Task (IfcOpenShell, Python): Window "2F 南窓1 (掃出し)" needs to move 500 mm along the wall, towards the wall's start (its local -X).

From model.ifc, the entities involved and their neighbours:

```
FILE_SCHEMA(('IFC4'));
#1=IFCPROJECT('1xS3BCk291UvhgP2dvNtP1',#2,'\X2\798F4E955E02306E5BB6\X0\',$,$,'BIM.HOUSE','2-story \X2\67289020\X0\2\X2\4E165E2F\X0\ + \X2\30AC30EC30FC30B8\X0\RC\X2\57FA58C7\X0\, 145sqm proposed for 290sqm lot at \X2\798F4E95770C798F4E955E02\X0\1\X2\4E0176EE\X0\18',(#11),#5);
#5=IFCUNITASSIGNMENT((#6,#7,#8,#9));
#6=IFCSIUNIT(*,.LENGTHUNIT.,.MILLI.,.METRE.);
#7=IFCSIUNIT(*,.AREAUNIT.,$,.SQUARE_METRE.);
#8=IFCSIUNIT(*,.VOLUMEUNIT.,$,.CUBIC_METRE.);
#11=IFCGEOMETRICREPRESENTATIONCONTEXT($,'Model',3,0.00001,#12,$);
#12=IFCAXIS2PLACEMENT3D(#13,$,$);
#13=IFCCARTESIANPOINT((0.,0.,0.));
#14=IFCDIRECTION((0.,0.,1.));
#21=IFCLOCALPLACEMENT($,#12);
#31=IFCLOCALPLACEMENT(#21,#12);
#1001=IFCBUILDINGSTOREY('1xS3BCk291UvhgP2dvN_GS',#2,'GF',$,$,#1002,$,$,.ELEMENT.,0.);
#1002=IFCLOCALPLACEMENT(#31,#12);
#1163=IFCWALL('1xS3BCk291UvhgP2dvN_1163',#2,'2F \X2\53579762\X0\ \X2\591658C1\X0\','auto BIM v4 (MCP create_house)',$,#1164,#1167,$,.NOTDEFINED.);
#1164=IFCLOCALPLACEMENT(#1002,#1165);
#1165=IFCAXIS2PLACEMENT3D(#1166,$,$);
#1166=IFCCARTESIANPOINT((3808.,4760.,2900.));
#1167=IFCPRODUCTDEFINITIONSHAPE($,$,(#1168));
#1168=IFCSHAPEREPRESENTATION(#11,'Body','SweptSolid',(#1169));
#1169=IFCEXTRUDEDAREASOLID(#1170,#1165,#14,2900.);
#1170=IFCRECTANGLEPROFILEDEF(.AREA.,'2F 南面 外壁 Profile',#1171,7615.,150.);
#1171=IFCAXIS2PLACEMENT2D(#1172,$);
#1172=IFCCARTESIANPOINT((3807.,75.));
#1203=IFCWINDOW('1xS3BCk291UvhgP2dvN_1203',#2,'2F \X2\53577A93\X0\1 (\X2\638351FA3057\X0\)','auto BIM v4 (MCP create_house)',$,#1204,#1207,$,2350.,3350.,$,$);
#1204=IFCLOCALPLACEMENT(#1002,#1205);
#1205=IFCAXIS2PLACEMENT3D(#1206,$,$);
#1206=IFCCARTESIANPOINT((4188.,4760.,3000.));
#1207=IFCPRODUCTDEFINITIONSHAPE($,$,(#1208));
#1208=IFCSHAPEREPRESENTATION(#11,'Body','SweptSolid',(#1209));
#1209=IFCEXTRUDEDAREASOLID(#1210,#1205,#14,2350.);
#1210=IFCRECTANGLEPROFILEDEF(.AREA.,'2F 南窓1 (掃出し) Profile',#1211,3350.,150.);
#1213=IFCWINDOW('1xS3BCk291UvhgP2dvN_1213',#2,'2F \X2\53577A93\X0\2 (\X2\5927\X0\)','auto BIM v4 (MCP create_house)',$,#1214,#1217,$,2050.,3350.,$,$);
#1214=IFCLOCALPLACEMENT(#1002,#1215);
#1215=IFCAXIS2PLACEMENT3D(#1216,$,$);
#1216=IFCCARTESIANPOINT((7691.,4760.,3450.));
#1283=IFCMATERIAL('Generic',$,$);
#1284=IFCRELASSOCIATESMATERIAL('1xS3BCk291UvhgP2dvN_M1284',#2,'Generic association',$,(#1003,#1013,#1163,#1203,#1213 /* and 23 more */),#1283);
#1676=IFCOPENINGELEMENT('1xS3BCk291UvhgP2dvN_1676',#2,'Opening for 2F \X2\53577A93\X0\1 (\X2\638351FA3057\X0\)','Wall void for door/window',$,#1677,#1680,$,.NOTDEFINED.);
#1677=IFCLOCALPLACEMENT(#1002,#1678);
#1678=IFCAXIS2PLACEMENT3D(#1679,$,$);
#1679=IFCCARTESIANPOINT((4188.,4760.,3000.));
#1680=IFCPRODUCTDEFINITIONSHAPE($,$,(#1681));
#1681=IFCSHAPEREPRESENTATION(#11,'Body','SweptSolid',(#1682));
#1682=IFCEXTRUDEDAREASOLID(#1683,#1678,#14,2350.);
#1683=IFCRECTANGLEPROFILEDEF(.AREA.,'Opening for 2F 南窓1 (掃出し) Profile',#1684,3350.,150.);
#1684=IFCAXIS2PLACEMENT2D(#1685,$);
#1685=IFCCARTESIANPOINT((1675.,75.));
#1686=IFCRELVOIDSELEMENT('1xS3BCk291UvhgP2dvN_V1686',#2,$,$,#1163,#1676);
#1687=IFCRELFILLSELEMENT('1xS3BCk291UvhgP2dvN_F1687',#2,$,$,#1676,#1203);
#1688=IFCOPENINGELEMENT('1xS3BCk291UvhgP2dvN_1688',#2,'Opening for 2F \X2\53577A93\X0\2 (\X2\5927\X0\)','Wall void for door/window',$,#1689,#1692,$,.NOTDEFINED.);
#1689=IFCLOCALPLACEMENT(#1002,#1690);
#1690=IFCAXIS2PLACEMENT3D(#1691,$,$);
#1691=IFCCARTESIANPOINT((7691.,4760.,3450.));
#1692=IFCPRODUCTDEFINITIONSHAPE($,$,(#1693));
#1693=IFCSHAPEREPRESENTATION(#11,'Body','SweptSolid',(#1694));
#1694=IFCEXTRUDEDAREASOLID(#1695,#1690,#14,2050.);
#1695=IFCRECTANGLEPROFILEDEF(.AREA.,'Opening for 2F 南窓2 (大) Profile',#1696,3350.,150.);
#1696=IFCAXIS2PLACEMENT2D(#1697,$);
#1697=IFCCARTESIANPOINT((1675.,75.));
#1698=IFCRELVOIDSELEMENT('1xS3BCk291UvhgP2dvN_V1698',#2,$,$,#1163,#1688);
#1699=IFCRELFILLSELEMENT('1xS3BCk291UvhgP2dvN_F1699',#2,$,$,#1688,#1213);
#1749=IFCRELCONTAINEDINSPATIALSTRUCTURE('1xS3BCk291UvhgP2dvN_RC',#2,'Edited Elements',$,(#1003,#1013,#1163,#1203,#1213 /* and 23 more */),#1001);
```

```python
import ifcopenshell
import ifcopenshell.api.geometry
import ifcopenshell.util.placement

model = ifcopenshell.open("model.ifc")

window = model.by_guid("1xS3BCk291UvhgP2dvN_1203")
opening = window.FillsVoids[0].RelatingOpeningElement
wall = opening.VoidsElements[0].RelatingBuildingElement

wall_matrix = ifcopenshell.util.placement.get_local_placement(wall.ObjectPlacement)
shift = wall_matrix[:3, 0] * -500.0
before = ifcopenshell.util.placement.get_local_placement(window.ObjectPlacement)[:3, 3].copy()

# The window is not placed relative to its opening, so move both.
for product in (opening, window):
    matrix = ifcopenshell.util.placement.get_local_placement(product.ObjectPlacement)
    matrix[:3, 3] += shift
    ifcopenshell.api.geometry.edit_object_placement(model, product=product, matrix=matrix, is_si=False)

after = ifcopenshell.util.placement.get_local_placement(window.ObjectPlacement)[:3, 3]
print("window moved by", (after - before).round(3) + 0.0)

model.write("model-out.ifc")
```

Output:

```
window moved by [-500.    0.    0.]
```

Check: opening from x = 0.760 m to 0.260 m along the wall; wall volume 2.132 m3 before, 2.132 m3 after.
